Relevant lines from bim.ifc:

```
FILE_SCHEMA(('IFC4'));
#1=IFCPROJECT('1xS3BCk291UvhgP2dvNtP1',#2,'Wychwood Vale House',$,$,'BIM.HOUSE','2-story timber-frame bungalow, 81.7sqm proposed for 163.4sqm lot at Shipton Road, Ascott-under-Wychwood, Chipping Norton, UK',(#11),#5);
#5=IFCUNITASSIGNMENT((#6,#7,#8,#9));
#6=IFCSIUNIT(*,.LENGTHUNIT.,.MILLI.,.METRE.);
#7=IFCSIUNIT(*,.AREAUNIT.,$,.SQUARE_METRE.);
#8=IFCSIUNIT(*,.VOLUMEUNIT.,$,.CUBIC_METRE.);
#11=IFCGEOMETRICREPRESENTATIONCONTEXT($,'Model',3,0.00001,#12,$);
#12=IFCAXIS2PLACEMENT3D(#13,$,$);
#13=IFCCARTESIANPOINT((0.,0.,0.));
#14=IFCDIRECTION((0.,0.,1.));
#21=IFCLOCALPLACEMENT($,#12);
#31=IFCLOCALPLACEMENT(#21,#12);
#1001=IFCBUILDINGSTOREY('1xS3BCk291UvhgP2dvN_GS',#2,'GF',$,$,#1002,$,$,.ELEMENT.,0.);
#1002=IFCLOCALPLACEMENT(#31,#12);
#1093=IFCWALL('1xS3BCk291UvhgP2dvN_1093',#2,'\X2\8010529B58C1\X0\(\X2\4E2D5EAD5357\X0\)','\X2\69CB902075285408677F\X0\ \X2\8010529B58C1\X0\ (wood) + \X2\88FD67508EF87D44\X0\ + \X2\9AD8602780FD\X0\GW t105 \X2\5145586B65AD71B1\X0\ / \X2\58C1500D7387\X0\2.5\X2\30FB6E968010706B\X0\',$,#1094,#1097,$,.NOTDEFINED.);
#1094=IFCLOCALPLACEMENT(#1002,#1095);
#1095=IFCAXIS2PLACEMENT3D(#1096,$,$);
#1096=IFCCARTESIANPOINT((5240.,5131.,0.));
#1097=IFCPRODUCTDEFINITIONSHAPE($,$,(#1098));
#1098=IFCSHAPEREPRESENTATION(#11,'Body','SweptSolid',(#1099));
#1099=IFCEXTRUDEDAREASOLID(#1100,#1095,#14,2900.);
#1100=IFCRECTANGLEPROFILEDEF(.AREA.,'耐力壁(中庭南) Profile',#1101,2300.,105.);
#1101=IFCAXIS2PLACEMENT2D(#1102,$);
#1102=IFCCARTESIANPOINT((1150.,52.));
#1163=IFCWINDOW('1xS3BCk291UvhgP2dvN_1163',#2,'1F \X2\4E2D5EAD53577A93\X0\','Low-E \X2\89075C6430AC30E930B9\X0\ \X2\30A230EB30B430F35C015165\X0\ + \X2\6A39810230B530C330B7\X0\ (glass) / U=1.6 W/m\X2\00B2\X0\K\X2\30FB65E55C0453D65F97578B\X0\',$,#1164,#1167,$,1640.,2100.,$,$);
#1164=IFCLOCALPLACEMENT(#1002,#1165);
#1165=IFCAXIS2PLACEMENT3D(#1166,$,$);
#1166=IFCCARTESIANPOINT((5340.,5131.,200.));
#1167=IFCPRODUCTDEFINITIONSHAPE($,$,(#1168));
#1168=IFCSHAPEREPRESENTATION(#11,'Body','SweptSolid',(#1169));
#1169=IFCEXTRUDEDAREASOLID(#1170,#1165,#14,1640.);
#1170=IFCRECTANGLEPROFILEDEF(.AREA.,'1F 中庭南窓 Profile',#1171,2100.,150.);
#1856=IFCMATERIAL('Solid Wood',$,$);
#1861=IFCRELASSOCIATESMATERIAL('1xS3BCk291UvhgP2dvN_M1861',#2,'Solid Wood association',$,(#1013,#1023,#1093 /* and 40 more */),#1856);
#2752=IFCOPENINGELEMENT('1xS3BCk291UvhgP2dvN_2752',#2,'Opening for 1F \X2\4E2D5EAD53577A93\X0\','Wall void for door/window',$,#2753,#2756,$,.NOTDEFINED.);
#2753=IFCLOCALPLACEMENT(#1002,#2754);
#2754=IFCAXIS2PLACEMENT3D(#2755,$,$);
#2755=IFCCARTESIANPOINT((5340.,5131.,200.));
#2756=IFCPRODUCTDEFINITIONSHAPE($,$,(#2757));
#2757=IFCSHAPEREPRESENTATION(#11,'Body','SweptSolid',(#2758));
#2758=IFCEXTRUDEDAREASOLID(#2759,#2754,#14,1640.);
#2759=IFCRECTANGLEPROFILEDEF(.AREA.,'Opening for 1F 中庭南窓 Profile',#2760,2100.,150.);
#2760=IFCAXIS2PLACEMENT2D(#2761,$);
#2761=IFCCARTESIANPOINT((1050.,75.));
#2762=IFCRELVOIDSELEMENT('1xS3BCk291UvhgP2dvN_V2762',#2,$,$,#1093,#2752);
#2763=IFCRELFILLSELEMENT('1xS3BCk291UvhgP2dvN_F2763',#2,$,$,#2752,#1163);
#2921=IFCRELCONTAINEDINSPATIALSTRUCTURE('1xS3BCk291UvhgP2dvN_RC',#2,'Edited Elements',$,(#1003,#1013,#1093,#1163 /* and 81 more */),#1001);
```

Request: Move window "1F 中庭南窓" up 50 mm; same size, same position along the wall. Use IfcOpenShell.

```python
import numpy as np
import ifcopenshell
import ifcopenshell.api.geometry
import ifcopenshell.util.placement
import ifcopenshell.util.unit

model = ifcopenshell.open("bim.ifc")
unit_scale = ifcopenshell.util.unit.calculate_unit_scale(model)

window = model.by_guid("1xS3BCk291UvhgP2dvN_1163")
opening = window.FillsVoids[0].RelatingOpeningElement
dz = 0.05 / unit_scale

shift = np.array([0.0, 0.0, dz])
# The window is not placed relative to its opening, so move both.
for product in (opening, window):
    matrix = ifcopenshell.util.placement.get_local_placement(product.ObjectPlacement)
    matrix[:3, 3] += shift
    ifcopenshell.api.geometry.edit_object_placement(model, product=product, matrix=matrix, is_si=False)

print(f"moved by {dz * unit_scale:+.3f} m")

model.write("bim_rev.ifc")
```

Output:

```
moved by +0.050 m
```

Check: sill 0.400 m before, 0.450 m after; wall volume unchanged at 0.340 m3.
